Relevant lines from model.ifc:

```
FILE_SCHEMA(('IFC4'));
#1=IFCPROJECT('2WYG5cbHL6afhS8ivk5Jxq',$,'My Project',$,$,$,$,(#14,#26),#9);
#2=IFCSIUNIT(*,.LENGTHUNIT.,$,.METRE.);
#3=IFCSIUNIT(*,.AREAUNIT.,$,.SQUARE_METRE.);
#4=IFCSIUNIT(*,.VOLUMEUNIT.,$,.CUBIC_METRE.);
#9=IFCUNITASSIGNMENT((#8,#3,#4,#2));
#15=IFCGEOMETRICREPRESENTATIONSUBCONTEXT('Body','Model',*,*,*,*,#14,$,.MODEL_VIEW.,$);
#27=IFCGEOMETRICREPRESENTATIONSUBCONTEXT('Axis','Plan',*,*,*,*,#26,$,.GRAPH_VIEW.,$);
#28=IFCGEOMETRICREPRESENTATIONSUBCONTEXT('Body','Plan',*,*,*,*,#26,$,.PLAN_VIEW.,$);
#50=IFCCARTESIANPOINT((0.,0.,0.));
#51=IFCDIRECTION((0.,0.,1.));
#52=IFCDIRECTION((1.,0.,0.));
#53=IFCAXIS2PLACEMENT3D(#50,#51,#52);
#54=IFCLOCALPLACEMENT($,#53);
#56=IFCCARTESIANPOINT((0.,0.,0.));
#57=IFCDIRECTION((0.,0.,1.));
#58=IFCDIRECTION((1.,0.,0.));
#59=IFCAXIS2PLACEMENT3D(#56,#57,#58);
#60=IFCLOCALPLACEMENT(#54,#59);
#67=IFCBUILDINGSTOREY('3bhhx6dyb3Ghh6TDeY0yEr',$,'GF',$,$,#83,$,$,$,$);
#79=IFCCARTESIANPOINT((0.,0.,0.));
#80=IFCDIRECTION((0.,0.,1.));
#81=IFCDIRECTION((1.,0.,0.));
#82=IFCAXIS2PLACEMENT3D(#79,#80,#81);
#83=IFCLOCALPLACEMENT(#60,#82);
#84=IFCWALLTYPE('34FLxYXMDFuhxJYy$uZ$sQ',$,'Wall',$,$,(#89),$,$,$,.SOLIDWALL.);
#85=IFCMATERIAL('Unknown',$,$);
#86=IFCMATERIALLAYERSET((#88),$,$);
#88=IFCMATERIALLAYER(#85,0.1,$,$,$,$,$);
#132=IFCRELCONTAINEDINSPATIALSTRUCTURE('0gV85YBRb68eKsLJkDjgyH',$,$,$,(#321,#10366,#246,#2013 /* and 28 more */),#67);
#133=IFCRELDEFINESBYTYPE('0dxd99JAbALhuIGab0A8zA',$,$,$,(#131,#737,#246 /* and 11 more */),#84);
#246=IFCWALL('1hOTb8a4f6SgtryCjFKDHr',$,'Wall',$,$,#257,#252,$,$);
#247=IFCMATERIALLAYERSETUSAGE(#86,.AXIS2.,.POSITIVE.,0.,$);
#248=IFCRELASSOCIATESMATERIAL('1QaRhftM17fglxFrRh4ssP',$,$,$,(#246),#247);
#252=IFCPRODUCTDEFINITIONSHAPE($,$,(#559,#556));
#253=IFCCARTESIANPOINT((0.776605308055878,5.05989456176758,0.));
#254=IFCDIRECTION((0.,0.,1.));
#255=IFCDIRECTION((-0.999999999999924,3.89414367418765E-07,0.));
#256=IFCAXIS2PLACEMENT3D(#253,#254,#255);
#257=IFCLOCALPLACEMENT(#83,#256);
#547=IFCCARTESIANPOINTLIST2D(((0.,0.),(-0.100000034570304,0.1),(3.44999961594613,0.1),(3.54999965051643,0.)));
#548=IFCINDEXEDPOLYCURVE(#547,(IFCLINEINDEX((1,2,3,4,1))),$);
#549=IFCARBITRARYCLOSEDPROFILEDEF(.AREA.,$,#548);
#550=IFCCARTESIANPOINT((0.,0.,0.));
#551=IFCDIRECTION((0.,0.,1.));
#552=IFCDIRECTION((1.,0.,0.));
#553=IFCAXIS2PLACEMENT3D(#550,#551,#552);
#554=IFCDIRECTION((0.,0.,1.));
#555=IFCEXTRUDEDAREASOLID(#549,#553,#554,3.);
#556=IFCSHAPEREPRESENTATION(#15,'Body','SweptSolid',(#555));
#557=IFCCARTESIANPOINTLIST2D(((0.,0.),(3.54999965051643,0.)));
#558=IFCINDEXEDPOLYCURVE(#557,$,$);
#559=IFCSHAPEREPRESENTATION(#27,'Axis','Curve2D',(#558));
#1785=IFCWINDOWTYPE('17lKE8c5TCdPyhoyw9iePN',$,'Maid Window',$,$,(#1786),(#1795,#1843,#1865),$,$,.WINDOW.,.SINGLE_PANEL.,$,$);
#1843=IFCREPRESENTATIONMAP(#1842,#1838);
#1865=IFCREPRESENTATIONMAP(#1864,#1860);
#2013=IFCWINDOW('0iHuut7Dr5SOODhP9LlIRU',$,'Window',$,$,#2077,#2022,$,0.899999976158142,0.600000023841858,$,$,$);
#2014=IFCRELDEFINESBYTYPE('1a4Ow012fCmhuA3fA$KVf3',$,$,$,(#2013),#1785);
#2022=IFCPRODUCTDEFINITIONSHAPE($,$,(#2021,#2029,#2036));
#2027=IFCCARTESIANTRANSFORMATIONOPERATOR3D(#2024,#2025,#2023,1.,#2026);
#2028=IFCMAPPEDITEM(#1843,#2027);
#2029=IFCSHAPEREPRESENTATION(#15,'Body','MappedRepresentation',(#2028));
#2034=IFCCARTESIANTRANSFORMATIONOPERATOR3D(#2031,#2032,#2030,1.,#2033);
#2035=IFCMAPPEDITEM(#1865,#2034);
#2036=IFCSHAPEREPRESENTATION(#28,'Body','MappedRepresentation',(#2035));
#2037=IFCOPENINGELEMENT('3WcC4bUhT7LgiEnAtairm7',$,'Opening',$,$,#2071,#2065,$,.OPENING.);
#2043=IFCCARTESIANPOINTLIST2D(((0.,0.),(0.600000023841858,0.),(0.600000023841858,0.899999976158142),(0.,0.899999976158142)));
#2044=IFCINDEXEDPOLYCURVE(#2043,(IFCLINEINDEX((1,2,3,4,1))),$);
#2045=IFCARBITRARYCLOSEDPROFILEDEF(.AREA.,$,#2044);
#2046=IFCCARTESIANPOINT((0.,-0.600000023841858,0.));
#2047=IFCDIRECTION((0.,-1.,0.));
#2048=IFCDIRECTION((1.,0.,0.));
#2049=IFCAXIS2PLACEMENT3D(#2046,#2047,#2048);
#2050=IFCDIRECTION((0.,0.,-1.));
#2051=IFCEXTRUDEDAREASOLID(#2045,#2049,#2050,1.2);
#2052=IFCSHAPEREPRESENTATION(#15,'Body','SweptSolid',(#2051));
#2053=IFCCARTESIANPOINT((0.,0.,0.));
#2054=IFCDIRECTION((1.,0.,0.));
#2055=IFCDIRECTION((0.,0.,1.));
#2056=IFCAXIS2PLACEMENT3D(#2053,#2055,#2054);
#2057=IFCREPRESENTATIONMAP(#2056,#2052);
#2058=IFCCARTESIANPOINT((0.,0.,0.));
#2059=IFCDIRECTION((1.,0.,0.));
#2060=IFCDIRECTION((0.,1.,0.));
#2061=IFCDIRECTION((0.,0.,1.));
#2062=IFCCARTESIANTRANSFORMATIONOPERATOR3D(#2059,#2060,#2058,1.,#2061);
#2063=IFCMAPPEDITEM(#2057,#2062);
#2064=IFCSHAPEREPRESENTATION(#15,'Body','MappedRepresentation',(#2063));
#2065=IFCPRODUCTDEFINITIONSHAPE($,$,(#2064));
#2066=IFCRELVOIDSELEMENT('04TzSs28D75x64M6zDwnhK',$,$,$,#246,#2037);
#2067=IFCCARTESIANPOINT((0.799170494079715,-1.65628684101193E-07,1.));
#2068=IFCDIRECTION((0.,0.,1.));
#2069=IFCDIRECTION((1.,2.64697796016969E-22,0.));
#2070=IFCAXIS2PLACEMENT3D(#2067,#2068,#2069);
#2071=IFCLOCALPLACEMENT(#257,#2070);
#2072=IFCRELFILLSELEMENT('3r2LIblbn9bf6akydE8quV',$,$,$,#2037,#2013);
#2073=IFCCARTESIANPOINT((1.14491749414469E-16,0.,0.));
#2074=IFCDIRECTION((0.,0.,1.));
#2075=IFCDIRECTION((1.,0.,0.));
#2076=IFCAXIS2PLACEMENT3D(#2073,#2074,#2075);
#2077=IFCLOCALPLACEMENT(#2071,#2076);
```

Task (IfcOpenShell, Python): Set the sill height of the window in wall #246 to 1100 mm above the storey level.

```python
import numpy as np
import ifcopenshell
import ifcopenshell.api.geometry
import ifcopenshell.geom
import ifcopenshell.util.element
import ifcopenshell.util.placement
import ifcopenshell.util.shape
import ifcopenshell.util.unit

model = ifcopenshell.open("model.ifc")
unit_scale = ifcopenshell.util.unit.calculate_unit_scale(model)

window = model.by_id(2013)
opening = window.FillsVoids[0].RelatingOpeningElement
storey = ifcopenshell.util.element.get_container(window, ifc_class="IfcBuildingStorey")
level = ifcopenshell.util.placement.get_local_placement(storey.ObjectPlacement)[2, 3]

# The opening's origin need not be at the sill, so measure its lowest point.
shape = ifcopenshell.geom.create_shape(ifcopenshell.geom.settings(), opening)
bottom = ifcopenshell.util.shape.get_shape_bottom_elevation(shape, shape.geometry) / unit_scale
dz = level + 1.1 / unit_scale - bottom

shift = np.array([0.0, 0.0, dz])
# The window is placed relative to its opening, so it follows when the opening moves.
matrix = ifcopenshell.util.placement.get_local_placement(opening.ObjectPlacement)
matrix[:3, 3] += shift
ifcopenshell.api.geometry.edit_object_placement(
    model, product=opening, matrix=matrix, is_si=False, should_transform_children=True
)

print(f"moved by {dz * unit_scale:+.3f} m")

model.write("model_edited.ifc")
```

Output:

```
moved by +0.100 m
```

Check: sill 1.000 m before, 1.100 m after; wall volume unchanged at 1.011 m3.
